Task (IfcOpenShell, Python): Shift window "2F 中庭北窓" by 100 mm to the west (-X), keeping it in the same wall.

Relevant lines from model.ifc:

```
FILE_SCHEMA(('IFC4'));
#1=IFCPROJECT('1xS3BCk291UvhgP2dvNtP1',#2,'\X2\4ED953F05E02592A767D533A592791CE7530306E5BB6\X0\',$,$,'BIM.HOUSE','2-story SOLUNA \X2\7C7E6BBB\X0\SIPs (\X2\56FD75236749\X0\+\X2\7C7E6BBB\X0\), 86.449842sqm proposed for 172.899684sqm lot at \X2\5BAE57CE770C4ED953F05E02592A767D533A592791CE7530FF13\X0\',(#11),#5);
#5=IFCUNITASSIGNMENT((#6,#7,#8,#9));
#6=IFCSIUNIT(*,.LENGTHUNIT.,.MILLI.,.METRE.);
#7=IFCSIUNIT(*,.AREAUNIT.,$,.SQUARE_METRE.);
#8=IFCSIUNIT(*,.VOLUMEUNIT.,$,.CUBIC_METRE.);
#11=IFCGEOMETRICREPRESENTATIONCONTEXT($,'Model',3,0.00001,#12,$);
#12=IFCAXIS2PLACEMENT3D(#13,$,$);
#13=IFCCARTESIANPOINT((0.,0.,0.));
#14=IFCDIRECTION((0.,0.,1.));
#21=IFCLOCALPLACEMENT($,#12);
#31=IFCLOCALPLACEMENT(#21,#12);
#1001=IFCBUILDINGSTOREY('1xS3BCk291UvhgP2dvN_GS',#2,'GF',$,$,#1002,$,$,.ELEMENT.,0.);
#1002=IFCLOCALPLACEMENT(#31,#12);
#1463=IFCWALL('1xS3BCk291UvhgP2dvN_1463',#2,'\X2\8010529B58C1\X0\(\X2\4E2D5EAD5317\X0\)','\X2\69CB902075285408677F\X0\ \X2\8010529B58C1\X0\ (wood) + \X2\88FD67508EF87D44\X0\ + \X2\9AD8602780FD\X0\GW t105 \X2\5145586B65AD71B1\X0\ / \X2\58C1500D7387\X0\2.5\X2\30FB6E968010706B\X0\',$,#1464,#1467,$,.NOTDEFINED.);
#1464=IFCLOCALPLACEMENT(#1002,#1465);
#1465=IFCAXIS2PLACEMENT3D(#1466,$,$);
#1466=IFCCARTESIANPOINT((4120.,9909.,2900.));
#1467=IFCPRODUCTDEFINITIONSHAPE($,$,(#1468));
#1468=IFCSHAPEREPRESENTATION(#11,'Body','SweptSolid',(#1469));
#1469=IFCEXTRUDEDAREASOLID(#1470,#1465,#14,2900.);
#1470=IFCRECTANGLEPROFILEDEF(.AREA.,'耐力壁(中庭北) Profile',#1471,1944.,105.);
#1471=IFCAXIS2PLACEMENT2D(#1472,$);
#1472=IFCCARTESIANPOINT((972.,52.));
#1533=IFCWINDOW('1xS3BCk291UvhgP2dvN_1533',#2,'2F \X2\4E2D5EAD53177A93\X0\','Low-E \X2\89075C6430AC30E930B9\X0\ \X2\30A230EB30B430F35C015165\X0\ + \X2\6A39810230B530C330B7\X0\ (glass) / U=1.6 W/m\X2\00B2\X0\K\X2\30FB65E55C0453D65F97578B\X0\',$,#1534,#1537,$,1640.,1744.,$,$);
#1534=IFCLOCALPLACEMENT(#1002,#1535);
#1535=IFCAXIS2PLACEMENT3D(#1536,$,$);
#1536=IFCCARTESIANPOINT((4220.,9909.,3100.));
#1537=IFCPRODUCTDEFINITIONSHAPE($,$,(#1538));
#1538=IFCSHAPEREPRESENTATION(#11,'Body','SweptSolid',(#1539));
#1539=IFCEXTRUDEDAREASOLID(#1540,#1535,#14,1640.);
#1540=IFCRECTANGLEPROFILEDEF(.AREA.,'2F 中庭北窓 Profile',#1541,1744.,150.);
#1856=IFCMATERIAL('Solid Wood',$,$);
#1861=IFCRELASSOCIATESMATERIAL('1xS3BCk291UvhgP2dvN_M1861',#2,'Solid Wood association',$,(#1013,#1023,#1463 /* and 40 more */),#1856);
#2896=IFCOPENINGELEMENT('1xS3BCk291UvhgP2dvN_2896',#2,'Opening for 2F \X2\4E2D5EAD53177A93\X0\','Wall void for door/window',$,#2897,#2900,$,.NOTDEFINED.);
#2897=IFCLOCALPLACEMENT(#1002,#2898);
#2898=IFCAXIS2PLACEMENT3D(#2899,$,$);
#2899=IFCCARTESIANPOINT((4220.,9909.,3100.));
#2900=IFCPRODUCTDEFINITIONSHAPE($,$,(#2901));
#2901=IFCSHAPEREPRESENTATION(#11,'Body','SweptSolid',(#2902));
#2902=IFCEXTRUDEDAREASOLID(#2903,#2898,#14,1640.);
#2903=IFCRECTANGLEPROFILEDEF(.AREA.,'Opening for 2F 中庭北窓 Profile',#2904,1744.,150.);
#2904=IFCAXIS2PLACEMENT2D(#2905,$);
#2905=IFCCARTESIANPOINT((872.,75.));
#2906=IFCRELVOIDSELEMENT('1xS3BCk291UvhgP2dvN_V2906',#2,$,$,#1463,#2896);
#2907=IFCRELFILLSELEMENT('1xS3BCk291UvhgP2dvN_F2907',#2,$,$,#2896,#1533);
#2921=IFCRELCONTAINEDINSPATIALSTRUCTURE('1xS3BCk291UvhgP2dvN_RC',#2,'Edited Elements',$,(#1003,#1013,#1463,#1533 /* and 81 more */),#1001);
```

```python
import ifcopenshell
import ifcopenshell.api.geometry
import ifcopenshell.util.placement

model = ifcopenshell.open("model.ifc")

window = model.by_guid("1xS3BCk291UvhgP2dvN_1533")
opening = window.FillsVoids[0].RelatingOpeningElement
wall = opening.VoidsElements[0].RelatingBuildingElement

wall_matrix = ifcopenshell.util.placement.get_local_placement(wall.ObjectPlacement)
shift = wall_matrix[:3, 0] * -100.0
before = ifcopenshell.util.placement.get_local_placement(window.ObjectPlacement)[:3, 3].copy()

# The window is not placed relative to its opening, so move both.
for product in (opening, window):
    matrix = ifcopenshell.util.placement.get_local_placement(product.ObjectPlacement)
    matrix[:3, 3] += shift
    ifcopenshell.api.geometry.edit_object_placement(model, product=product, matrix=matrix, is_si=False)

after = ifcopenshell.util.placement.get_local_placement(window.ObjectPlacement)[:3, 3]
print("window moved by", (after - before).round(3) + 0.0)

model.write("model_v2.ifc")
```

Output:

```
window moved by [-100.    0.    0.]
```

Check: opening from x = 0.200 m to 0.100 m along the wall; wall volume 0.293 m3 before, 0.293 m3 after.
